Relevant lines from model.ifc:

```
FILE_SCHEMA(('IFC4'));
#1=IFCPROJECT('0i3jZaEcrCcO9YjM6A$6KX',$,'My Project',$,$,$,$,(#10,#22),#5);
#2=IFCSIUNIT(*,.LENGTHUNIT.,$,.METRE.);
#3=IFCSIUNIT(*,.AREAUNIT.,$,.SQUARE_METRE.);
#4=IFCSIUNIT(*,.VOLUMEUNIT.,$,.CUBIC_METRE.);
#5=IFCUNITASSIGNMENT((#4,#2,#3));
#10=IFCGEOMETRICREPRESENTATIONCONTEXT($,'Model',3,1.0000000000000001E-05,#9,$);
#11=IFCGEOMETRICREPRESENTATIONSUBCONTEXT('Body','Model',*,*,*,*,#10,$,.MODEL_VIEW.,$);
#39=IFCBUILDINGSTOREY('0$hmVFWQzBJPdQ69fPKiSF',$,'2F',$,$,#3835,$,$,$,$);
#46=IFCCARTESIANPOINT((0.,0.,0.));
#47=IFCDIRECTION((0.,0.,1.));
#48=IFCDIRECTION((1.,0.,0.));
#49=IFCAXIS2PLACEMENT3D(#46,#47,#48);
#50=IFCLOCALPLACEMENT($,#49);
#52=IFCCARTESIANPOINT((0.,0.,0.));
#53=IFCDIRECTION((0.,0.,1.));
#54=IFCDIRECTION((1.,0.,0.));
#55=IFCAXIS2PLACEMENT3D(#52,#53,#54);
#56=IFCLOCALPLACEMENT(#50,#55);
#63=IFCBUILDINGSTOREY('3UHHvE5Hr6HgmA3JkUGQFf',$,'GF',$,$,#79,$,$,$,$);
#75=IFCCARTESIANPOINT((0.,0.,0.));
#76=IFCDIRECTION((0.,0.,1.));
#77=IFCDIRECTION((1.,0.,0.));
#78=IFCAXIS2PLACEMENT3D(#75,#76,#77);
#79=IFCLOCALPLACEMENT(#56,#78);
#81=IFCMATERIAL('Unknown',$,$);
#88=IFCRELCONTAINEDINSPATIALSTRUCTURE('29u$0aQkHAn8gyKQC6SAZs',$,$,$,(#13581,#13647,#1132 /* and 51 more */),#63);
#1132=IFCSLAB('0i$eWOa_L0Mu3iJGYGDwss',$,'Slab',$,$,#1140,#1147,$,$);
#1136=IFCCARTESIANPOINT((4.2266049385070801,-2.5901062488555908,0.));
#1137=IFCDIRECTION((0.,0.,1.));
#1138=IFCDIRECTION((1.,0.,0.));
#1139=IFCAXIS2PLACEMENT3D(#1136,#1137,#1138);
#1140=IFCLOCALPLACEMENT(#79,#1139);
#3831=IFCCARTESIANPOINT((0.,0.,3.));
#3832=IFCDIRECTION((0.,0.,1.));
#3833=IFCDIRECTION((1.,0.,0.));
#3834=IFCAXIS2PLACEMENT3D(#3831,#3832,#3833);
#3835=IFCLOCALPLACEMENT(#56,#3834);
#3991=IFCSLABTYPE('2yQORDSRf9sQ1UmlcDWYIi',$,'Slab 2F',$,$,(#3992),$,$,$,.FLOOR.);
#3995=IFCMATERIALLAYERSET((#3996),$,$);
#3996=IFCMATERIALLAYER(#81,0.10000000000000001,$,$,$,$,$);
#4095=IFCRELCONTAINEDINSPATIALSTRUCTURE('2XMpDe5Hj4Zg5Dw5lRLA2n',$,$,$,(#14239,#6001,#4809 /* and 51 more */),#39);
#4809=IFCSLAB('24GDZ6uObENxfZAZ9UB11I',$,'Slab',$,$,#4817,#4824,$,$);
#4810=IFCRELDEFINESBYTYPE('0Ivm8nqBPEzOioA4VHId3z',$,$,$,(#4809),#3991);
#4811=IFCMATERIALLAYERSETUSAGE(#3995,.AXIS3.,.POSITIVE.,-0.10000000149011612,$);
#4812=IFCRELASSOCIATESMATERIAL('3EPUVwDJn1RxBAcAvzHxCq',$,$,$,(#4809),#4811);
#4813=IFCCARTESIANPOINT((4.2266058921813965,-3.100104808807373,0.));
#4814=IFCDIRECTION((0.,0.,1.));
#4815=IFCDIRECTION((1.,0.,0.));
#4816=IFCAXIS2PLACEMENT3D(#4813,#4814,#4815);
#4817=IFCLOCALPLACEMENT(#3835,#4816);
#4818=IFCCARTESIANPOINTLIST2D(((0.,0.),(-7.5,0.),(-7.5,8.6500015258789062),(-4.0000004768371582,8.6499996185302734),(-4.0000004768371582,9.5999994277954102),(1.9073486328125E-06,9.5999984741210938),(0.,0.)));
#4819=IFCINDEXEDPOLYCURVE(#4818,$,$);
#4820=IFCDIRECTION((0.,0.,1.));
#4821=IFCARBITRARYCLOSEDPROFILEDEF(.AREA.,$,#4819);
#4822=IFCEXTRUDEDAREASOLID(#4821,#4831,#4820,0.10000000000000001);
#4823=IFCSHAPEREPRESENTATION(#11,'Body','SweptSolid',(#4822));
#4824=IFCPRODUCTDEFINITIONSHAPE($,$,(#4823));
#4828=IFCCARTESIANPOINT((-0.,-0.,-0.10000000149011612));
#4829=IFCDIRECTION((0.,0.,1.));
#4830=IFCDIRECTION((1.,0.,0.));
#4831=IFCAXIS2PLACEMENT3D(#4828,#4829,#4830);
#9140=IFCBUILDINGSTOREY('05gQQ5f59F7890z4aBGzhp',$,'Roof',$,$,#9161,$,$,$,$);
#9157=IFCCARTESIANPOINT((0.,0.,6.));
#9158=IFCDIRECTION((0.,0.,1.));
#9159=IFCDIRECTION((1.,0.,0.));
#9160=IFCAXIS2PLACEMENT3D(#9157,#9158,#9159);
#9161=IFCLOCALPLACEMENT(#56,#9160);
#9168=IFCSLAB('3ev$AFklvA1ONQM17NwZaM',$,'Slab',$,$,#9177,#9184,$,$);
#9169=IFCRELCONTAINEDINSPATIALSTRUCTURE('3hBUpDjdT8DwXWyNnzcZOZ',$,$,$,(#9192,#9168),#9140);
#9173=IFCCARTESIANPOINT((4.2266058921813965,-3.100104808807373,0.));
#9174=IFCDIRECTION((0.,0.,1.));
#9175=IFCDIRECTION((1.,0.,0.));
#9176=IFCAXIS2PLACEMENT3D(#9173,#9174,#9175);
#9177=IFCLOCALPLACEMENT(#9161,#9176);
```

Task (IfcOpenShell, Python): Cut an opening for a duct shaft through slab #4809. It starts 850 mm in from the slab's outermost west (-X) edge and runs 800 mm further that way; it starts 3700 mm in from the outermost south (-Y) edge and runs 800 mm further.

```python
import numpy as np
import ifcopenshell
import ifcopenshell.api.feature
import ifcopenshell.api.geometry
import ifcopenshell.api.root
import ifcopenshell.geom
import ifcopenshell.util.placement
import ifcopenshell.util.representation
import ifcopenshell.util.shape
import ifcopenshell.util.unit

model = ifcopenshell.open("model.ifc")
unit_scale = ifcopenshell.util.unit.calculate_unit_scale(model)
settings = ifcopenshell.geom.settings()


def volume(element):
    """Net volume in cubic metres, openings subtracted."""
    shape = ifcopenshell.geom.create_shape(settings, element)
    return ifcopenshell.util.shape.get_volume(shape.geometry)


slab = model.by_guid("24GDZ6uObENxfZAZ9UB11I")
before = volume(slab)

# Extent in the slab's own axes, in metres. The edges named are its -X and -Y sides.
slab_shape = ifcopenshell.geom.create_shape(settings, slab)
vertices = ifcopenshell.util.shape.get_vertices(slab_shape.geometry)
x_min, y_min, bottom = vertices.min(axis=0)
top = vertices[:, 2].max()

opening = ifcopenshell.api.root.create_entity(model, ifc_class="IfcOpeningElement", name="Duct shaft opening", predefined_type="OPENING")
context = ifcopenshell.util.representation.get_context(model, "Model", "Body", "MODEL_VIEW")
width, depth = 0.8, 0.8
outline = [(0.0, 0.0), (width, 0.0), (width, depth), (0.0, depth), (0.0, 0.0)]
# Overshoot both faces by 50 mm so the cut is clean.
shape = ifcopenshell.api.geometry.add_slab_representation(
    model, context=context, depth=top - bottom + 0.1, polyline=outline
)
ifcopenshell.api.geometry.assign_representation(model, product=opening, representation=shape)

matrix = ifcopenshell.util.placement.get_local_placement(slab.ObjectPlacement)
matrix[:, 3] = matrix @ np.append(np.array([x_min + 0.85, y_min + 3.7, bottom - 0.05]) / unit_scale, 1.0)
ifcopenshell.api.geometry.edit_object_placement(model, product=opening, matrix=matrix, is_si=False)
ifcopenshell.api.feature.add_feature(model, feature=opening, element=slab)

after = volume(slab)

print(f"slab volume {before:.3f} -> {after:.3f} m3")

model.write("model-out.ifc")
```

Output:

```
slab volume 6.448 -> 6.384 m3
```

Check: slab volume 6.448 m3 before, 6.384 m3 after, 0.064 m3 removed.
